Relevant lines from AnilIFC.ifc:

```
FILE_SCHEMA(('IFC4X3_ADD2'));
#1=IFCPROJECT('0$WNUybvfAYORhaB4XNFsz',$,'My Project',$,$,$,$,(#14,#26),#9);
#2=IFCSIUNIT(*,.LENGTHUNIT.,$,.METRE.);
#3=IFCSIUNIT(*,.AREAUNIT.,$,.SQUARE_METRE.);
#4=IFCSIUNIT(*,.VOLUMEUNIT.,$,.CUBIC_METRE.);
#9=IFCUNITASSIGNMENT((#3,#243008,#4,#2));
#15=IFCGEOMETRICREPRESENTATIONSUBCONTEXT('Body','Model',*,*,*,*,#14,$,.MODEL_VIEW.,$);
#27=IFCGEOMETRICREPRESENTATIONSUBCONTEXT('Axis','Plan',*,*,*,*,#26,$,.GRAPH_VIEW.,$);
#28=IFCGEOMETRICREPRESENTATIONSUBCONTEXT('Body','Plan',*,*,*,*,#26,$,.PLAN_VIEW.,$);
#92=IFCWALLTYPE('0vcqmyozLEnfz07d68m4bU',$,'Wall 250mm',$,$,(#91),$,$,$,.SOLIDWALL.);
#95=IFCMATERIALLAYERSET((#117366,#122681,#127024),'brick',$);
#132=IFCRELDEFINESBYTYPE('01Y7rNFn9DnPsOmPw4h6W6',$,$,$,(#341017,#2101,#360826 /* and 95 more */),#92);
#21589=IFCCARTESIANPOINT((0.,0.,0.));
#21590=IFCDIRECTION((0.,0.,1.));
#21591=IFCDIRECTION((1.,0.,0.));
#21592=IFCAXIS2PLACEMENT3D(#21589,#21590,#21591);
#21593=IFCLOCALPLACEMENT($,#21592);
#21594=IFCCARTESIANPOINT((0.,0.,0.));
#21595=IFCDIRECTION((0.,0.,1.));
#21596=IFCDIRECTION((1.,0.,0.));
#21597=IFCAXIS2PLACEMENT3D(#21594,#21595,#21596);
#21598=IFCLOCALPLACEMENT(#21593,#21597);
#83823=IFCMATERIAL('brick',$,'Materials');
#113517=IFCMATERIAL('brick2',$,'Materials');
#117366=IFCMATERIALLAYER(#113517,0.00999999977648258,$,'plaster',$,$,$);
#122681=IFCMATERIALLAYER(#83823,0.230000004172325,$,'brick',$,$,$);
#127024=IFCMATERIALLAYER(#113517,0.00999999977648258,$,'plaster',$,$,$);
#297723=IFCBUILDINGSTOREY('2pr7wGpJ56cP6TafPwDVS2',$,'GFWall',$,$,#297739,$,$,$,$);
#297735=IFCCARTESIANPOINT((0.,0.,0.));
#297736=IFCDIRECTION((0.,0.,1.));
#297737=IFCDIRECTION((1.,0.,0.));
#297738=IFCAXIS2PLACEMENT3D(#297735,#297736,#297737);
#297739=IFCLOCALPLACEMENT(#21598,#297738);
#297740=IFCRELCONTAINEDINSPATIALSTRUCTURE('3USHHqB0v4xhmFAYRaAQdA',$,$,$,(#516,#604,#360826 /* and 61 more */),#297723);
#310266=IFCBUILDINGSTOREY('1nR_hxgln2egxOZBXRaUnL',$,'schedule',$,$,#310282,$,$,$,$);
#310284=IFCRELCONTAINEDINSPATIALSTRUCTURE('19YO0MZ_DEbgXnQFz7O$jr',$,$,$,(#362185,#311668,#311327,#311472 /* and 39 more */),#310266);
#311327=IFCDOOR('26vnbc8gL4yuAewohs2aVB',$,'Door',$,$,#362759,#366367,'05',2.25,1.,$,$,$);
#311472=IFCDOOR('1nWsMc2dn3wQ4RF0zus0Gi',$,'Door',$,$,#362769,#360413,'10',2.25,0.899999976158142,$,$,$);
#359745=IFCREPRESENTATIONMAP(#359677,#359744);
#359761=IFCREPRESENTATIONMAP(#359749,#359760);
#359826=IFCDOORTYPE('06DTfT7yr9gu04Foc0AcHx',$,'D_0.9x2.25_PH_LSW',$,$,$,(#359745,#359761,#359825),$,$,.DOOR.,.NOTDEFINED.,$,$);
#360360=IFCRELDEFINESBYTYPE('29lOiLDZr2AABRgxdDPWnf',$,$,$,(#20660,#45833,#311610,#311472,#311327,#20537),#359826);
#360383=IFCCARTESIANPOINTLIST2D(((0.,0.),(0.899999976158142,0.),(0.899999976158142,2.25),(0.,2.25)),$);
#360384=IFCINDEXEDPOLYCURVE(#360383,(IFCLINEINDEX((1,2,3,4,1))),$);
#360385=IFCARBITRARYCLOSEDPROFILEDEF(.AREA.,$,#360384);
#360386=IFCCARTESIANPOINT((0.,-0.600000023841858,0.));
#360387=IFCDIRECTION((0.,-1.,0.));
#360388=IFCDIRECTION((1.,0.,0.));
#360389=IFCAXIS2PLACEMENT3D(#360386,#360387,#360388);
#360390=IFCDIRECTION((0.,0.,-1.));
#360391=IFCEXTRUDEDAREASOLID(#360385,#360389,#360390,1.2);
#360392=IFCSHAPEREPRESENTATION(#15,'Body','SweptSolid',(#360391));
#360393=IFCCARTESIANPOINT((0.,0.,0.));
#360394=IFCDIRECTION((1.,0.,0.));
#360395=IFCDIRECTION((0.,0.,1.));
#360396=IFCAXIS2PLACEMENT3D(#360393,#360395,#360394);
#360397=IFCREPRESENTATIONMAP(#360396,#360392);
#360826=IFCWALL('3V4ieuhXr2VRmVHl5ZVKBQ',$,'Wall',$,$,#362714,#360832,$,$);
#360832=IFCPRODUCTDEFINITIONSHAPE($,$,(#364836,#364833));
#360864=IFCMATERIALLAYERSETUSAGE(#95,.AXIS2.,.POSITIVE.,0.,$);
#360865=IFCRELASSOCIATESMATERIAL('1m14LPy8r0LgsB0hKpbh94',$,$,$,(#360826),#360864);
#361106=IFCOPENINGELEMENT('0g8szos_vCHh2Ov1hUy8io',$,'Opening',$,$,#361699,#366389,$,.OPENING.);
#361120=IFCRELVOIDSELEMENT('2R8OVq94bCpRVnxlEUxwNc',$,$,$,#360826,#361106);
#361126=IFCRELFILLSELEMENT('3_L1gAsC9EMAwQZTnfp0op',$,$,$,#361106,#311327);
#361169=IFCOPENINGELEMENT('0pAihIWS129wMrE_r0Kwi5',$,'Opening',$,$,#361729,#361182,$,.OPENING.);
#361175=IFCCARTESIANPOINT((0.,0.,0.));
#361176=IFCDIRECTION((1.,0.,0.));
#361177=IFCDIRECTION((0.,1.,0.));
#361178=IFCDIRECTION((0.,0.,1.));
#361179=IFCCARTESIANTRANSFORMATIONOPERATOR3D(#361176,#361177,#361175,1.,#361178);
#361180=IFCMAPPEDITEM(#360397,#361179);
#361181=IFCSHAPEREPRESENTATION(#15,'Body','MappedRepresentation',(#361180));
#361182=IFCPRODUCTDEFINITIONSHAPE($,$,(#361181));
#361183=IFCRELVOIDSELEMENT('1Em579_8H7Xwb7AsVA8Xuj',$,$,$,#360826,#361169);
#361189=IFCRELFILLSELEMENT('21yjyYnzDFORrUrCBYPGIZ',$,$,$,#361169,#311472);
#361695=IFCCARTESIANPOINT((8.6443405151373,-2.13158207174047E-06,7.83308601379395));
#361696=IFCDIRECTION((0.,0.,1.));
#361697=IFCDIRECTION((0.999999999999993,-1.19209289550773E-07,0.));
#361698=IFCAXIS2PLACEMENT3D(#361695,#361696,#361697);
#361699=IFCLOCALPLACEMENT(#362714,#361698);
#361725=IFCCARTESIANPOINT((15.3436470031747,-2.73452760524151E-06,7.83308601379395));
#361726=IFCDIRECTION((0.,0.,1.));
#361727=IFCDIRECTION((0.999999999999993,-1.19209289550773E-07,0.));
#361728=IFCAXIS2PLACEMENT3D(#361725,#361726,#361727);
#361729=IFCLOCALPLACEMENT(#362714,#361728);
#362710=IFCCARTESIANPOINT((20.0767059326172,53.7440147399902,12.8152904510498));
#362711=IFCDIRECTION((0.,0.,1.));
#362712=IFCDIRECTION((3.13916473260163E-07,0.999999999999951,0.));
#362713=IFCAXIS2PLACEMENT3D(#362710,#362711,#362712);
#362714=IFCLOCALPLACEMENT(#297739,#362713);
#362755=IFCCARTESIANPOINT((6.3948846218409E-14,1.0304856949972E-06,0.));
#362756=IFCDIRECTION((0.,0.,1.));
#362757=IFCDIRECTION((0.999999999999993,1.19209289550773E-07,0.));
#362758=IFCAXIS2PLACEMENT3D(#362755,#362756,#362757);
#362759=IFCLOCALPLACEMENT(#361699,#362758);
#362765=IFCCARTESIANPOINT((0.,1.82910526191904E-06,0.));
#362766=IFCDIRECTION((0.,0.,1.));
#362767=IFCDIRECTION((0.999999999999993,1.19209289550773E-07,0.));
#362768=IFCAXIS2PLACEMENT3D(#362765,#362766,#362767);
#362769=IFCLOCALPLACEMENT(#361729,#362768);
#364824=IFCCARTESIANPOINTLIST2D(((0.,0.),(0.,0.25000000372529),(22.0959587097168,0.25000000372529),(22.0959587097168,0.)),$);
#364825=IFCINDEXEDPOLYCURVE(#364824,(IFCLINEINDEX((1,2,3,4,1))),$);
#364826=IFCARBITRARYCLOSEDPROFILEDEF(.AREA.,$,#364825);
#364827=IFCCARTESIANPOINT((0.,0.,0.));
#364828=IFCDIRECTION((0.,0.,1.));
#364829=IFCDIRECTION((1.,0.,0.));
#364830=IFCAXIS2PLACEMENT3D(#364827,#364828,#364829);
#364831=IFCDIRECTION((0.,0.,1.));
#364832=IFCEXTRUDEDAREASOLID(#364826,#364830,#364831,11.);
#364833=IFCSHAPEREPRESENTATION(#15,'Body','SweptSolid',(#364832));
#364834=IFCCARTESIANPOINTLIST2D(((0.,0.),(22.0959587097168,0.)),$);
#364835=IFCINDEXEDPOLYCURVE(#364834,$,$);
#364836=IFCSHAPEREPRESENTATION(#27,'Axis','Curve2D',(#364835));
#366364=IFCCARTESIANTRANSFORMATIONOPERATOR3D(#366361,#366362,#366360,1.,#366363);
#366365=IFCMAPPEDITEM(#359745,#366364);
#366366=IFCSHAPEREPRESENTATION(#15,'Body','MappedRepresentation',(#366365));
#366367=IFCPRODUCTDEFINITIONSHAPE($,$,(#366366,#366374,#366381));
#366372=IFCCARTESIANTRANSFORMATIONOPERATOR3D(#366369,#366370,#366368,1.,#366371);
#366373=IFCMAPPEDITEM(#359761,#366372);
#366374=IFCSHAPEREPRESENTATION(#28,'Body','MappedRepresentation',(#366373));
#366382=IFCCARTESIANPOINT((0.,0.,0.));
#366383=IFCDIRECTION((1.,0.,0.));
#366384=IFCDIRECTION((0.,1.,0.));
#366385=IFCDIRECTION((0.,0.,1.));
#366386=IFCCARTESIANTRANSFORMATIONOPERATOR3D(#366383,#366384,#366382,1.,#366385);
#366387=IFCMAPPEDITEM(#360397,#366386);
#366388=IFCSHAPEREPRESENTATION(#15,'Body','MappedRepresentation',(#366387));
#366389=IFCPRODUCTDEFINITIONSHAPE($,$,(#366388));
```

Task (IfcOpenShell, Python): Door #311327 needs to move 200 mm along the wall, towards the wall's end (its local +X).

```python
import ifcopenshell
import ifcopenshell.api.geometry
import ifcopenshell.util.placement

model = ifcopenshell.open("AnilIFC.ifc")

door = model.by_guid("26vnbc8gL4yuAewohs2aVB")
opening = door.FillsVoids[0].RelatingOpeningElement
wall = opening.VoidsElements[0].RelatingBuildingElement

wall_matrix = ifcopenshell.util.placement.get_local_placement(wall.ObjectPlacement)
shift = wall_matrix[:3, 0] * 0.2
before = ifcopenshell.util.placement.get_local_placement(door.ObjectPlacement)[:3, 3].copy()

# The door is placed relative to its opening, so it follows when the opening moves.
matrix = ifcopenshell.util.placement.get_local_placement(opening.ObjectPlacement)
matrix[:3, 3] += shift
ifcopenshell.api.geometry.edit_object_placement(
    model, product=opening, matrix=matrix, is_si=False, should_transform_children=True
)

after = ifcopenshell.util.placement.get_local_placement(door.ObjectPlacement)[:3, 3]
print("door moved by", (after - before).round(3) + 0.0)

model.write("AnilIFC-out.ifc")
```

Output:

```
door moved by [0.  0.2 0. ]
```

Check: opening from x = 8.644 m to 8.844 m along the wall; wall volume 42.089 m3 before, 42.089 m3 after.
